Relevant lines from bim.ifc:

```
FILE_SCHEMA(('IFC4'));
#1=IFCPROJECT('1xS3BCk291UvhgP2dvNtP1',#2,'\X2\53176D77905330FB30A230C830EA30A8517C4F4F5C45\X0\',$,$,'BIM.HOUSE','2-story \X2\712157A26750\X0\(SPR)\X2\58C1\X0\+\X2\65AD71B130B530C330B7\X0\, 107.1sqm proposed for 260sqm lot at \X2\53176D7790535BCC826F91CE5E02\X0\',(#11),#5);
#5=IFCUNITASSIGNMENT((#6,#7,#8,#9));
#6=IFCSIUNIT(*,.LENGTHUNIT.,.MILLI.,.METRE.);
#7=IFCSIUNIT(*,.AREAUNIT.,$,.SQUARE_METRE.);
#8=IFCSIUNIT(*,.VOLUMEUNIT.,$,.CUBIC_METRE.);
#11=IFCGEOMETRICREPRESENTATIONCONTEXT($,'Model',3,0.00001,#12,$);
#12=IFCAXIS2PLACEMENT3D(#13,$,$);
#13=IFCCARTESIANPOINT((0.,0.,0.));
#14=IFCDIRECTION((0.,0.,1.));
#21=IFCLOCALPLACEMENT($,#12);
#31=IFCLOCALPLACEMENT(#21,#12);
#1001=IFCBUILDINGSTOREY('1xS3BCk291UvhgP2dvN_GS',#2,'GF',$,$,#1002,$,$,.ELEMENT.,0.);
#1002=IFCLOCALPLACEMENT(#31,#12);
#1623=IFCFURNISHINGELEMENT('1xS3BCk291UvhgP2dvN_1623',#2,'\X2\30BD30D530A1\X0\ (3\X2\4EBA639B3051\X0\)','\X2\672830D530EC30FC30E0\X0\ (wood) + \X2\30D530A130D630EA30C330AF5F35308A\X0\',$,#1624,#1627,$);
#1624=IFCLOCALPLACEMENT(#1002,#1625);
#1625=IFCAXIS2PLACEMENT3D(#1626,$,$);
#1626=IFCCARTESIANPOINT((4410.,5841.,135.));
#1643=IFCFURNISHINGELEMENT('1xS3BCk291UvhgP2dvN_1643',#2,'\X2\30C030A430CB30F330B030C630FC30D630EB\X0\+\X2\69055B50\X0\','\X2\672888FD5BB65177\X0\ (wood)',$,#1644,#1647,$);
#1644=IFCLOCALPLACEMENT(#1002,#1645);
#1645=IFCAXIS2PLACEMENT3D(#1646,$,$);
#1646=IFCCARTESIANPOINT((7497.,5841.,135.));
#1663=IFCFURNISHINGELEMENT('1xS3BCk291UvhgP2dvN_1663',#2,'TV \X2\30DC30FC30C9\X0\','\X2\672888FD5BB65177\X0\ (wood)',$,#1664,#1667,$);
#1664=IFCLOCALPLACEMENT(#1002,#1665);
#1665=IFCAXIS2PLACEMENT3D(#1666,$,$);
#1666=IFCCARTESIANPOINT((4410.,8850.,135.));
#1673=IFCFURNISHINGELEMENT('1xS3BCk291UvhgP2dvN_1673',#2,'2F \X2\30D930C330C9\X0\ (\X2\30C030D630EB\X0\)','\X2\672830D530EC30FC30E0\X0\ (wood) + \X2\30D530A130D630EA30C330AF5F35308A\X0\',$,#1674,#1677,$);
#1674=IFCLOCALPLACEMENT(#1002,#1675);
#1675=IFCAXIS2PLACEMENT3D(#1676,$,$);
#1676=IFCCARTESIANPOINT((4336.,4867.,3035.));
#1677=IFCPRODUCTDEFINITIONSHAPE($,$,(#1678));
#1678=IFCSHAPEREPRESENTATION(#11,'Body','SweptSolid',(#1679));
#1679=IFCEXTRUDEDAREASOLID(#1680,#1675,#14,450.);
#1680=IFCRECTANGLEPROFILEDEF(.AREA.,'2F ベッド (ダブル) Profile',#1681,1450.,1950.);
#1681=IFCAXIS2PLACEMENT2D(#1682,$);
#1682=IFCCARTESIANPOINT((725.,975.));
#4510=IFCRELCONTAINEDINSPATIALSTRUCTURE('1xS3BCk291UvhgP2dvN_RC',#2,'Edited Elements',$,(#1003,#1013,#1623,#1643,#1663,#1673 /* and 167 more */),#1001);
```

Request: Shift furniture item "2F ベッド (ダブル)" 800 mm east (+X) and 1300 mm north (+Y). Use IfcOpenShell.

```python
import ifcopenshell
import ifcopenshell.api.geometry
import ifcopenshell.util.placement
import ifcopenshell.util.unit

model = ifcopenshell.open("bim.ifc")
unit_scale = ifcopenshell.util.unit.calculate_unit_scale(model)

item = model.by_id(1673)
matrix = ifcopenshell.util.placement.get_local_placement(item.ObjectPlacement)
matrix[0, 3] += 0.8 / unit_scale
matrix[1, 3] += 1.3 / unit_scale
ifcopenshell.api.geometry.edit_object_placement(model, product=item, matrix=matrix, is_si=False)

print(ifcopenshell.util.placement.get_local_placement(item.ObjectPlacement).round(3) + 0.0)

model.write("bim_updated.ifc")
```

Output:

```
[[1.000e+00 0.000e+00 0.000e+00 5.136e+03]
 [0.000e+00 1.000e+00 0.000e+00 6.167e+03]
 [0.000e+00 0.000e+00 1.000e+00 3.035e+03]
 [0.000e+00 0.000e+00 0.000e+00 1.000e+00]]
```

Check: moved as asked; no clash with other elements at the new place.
